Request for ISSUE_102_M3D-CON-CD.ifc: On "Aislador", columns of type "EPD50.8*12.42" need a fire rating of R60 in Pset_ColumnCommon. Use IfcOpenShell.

First a look at what the model holds.

```python
import ifcopenshell
import ifcopenshell.util.element

model = ifcopenshell.open("ISSUE_102_M3D-CON-CD.ifc")
print(model.schema)
storey = next(s for s in model.by_type("IfcBuildingStorey") if s.Name == "Aislador")
columns = [e for e in ifcopenshell.util.element.get_decomposition(storey) if e.is_a("IfcColumn")]
seen = {}
for e in columns:
    element_type = ifcopenshell.util.element.get_type(e)
    key = (element_type.Name if element_type != e and element_type else None, ifcopenshell.util.element.get_pset(e, "Pset_ColumnCommon", "FireRating"))
    seen[key] = seen.get(key, 0) + 1
for (name, value), count in sorted(seen.items(), key=str):
    print(count, "x", name, "|", value)
```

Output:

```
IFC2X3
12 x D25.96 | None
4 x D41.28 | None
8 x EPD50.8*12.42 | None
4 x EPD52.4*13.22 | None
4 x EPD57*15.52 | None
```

```python
import ifcopenshell
import ifcopenshell.api.pset
import ifcopenshell.util.element

model = ifcopenshell.open("ISSUE_102_M3D-CON-CD.ifc")

storey = next(s for s in model.by_type("IfcBuildingStorey") if s.Name == "Aislador")
columns = [e for e in ifcopenshell.util.element.get_decomposition(storey) if e.is_a("IfcColumn")]

count = 0
for e in columns:
    element_type = ifcopenshell.util.element.get_type(e)
    if element_type in (None, e) or element_type.Name != "EPD50.8*12.42":
        continue
    found = ifcopenshell.util.element.get_pset(e, "Pset_ColumnCommon", should_inherit=False)
    if found:
        pset = model.by_id(found["id"])
        if len(ifcopenshell.util.element.get_elements_by_pset(pset)) > 1:
            pset = ifcopenshell.api.pset.unshare_pset(model, products=[e], pset=pset)[0]
    else:
        pset = ifcopenshell.api.pset.add_pset(model, product=e, name="Pset_ColumnCommon")
    ifcopenshell.api.pset.edit_pset(model, pset=pset, properties={"FireRating": "R60"})
    count += 1

print(count, "columns updated")

model.write("ISSUE_102_M3D-CON-CD_v2.ifc")
```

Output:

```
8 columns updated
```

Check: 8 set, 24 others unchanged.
